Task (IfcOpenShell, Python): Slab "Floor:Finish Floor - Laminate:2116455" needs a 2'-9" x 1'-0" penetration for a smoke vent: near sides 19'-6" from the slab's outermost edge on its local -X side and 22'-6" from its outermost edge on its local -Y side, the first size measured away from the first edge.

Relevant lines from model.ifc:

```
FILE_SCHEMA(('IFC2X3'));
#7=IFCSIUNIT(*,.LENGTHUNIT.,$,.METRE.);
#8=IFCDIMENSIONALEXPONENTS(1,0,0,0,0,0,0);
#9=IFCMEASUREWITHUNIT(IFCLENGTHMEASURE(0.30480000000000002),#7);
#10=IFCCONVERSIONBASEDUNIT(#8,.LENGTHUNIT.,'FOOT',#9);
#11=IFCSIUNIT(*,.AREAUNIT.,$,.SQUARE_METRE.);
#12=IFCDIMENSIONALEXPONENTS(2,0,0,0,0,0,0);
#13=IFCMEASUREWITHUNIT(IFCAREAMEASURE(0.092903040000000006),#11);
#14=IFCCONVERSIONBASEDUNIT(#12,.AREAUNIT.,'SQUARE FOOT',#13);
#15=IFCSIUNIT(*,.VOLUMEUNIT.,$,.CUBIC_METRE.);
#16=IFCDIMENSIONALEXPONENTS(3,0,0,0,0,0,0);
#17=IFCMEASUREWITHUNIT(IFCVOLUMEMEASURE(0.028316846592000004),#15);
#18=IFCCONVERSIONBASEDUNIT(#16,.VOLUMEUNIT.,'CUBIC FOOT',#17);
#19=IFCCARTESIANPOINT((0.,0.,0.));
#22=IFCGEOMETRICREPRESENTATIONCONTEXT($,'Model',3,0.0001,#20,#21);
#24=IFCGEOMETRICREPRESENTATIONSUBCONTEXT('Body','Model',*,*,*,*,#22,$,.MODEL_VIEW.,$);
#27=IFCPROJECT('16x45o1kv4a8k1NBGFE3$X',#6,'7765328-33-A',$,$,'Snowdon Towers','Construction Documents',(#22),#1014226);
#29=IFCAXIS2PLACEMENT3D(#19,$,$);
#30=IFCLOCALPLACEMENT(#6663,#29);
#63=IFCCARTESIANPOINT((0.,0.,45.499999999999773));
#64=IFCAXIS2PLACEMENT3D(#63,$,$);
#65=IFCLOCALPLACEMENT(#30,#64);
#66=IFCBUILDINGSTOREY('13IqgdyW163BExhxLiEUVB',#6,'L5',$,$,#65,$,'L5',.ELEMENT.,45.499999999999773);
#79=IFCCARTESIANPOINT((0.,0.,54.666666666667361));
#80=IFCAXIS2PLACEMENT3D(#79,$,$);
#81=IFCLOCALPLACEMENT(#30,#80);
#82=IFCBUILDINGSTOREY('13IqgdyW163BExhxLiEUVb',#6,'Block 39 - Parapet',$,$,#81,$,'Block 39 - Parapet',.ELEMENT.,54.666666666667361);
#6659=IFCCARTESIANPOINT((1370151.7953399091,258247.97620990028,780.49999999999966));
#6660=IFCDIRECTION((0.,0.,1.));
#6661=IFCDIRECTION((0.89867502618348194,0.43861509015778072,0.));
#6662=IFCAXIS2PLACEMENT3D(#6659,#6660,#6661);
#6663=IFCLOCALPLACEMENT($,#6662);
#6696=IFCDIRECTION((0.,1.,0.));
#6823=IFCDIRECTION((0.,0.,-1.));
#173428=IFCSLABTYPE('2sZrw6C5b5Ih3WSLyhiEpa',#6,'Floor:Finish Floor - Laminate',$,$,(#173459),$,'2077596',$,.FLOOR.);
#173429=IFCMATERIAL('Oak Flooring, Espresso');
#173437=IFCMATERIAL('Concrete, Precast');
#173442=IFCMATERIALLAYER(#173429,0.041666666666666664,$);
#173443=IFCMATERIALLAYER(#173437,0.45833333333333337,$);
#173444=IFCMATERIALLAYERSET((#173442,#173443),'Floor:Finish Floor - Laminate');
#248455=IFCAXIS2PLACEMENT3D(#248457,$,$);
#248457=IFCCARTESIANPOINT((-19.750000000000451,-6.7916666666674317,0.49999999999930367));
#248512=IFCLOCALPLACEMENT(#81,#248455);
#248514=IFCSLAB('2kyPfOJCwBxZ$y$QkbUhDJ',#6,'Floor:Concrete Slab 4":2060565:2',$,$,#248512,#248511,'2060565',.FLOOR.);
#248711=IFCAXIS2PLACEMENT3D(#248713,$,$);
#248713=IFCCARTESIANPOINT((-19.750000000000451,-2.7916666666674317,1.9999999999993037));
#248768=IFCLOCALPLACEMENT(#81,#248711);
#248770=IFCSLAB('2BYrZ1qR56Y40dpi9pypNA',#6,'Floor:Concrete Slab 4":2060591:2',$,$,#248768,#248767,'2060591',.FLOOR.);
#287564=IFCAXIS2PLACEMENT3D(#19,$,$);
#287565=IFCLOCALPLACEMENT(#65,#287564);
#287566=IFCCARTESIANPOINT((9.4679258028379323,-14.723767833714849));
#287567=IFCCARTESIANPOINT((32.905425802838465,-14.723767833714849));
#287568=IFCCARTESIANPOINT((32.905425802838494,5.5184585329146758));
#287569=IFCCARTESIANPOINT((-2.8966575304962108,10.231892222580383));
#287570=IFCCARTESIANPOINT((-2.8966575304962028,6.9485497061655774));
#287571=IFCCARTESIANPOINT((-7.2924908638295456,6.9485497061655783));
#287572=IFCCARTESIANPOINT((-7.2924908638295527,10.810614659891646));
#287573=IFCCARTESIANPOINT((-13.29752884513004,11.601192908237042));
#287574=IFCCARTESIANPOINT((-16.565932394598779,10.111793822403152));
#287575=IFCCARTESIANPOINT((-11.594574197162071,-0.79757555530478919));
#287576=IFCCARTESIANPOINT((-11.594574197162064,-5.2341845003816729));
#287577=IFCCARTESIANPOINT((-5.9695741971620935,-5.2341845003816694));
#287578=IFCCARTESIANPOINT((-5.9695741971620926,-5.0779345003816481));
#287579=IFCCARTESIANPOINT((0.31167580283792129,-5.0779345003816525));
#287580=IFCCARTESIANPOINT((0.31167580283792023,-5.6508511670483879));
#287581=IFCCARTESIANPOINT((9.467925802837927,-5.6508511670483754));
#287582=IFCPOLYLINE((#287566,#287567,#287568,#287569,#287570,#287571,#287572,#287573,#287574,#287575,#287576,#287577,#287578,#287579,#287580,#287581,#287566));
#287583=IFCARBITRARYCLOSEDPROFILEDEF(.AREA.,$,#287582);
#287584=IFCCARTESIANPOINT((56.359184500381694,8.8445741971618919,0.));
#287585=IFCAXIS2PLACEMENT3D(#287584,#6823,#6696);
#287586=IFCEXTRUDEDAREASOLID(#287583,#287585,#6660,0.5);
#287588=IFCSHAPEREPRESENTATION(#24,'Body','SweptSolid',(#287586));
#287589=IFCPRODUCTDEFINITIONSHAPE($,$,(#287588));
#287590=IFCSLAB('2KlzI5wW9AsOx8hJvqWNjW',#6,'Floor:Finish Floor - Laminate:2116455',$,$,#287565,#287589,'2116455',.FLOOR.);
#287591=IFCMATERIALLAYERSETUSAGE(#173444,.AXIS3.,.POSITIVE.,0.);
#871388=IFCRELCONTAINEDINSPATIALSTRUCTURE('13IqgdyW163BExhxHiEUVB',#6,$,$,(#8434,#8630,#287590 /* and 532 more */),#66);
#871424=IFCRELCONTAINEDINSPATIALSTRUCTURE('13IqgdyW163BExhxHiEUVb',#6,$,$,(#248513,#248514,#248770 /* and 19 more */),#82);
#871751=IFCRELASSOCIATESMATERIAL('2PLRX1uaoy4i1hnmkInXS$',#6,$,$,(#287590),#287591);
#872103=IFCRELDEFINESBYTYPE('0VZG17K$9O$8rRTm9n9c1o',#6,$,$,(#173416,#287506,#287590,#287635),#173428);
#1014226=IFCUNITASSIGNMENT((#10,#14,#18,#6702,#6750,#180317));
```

```python
import numpy as np
import ifcopenshell
import ifcopenshell.api.feature
import ifcopenshell.api.geometry
import ifcopenshell.api.root
import ifcopenshell.geom
import ifcopenshell.util.placement
import ifcopenshell.util.representation
import ifcopenshell.util.shape
import ifcopenshell.util.unit

model = ifcopenshell.open("model.ifc")
unit_scale = ifcopenshell.util.unit.calculate_unit_scale(model)
settings = ifcopenshell.geom.settings()


def volume(element):
    """Net volume in cubic metres, openings subtracted."""
    shape = ifcopenshell.geom.create_shape(settings, element)
    return ifcopenshell.util.shape.get_volume(shape.geometry)


slab = model.by_id(287590)
before = volume(slab)

# Extent in the slab's own axes, in metres. The edges named are its -X and -Y sides.
slab_shape = ifcopenshell.geom.create_shape(settings, slab)
vertices = ifcopenshell.util.shape.get_vertices(slab_shape.geometry)
x_min, y_min, bottom = vertices.min(axis=0)
top = vertices[:, 2].max()

opening = ifcopenshell.api.root.create_entity(model, ifc_class="IfcOpeningElement", name="Smoke vent opening")
context = ifcopenshell.util.representation.get_context(model, "Model", "Body", "MODEL_VIEW")
width, depth = 0.8382, 0.3048
outline = [(0.0, 0.0), (width, 0.0), (width, depth), (0.0, depth), (0.0, 0.0)]
# Overshoot both faces by 50 mm so the cut is clean.
shape = ifcopenshell.api.geometry.add_slab_representation(
    model, context=context, depth=top - bottom + 0.1, polyline=outline
)
ifcopenshell.api.geometry.assign_representation(model, product=opening, representation=shape)

matrix = ifcopenshell.util.placement.get_local_placement(slab.ObjectPlacement)
matrix[:, 3] = matrix @ np.append(np.array([x_min + 5.9436, y_min + 6.858, bottom - 0.05]) / unit_scale, 1.0)
ifcopenshell.api.geometry.edit_object_placement(model, product=opening, matrix=matrix, is_si=False)
ifcopenshell.api.feature.add_feature(model, feature=opening, element=slab)

after = volume(slab)

print(f"slab volume {before:.3f} -> {after:.3f} m3")

model.write("model_updated.ifc")
```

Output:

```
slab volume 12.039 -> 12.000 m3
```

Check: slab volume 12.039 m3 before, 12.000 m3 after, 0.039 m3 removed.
